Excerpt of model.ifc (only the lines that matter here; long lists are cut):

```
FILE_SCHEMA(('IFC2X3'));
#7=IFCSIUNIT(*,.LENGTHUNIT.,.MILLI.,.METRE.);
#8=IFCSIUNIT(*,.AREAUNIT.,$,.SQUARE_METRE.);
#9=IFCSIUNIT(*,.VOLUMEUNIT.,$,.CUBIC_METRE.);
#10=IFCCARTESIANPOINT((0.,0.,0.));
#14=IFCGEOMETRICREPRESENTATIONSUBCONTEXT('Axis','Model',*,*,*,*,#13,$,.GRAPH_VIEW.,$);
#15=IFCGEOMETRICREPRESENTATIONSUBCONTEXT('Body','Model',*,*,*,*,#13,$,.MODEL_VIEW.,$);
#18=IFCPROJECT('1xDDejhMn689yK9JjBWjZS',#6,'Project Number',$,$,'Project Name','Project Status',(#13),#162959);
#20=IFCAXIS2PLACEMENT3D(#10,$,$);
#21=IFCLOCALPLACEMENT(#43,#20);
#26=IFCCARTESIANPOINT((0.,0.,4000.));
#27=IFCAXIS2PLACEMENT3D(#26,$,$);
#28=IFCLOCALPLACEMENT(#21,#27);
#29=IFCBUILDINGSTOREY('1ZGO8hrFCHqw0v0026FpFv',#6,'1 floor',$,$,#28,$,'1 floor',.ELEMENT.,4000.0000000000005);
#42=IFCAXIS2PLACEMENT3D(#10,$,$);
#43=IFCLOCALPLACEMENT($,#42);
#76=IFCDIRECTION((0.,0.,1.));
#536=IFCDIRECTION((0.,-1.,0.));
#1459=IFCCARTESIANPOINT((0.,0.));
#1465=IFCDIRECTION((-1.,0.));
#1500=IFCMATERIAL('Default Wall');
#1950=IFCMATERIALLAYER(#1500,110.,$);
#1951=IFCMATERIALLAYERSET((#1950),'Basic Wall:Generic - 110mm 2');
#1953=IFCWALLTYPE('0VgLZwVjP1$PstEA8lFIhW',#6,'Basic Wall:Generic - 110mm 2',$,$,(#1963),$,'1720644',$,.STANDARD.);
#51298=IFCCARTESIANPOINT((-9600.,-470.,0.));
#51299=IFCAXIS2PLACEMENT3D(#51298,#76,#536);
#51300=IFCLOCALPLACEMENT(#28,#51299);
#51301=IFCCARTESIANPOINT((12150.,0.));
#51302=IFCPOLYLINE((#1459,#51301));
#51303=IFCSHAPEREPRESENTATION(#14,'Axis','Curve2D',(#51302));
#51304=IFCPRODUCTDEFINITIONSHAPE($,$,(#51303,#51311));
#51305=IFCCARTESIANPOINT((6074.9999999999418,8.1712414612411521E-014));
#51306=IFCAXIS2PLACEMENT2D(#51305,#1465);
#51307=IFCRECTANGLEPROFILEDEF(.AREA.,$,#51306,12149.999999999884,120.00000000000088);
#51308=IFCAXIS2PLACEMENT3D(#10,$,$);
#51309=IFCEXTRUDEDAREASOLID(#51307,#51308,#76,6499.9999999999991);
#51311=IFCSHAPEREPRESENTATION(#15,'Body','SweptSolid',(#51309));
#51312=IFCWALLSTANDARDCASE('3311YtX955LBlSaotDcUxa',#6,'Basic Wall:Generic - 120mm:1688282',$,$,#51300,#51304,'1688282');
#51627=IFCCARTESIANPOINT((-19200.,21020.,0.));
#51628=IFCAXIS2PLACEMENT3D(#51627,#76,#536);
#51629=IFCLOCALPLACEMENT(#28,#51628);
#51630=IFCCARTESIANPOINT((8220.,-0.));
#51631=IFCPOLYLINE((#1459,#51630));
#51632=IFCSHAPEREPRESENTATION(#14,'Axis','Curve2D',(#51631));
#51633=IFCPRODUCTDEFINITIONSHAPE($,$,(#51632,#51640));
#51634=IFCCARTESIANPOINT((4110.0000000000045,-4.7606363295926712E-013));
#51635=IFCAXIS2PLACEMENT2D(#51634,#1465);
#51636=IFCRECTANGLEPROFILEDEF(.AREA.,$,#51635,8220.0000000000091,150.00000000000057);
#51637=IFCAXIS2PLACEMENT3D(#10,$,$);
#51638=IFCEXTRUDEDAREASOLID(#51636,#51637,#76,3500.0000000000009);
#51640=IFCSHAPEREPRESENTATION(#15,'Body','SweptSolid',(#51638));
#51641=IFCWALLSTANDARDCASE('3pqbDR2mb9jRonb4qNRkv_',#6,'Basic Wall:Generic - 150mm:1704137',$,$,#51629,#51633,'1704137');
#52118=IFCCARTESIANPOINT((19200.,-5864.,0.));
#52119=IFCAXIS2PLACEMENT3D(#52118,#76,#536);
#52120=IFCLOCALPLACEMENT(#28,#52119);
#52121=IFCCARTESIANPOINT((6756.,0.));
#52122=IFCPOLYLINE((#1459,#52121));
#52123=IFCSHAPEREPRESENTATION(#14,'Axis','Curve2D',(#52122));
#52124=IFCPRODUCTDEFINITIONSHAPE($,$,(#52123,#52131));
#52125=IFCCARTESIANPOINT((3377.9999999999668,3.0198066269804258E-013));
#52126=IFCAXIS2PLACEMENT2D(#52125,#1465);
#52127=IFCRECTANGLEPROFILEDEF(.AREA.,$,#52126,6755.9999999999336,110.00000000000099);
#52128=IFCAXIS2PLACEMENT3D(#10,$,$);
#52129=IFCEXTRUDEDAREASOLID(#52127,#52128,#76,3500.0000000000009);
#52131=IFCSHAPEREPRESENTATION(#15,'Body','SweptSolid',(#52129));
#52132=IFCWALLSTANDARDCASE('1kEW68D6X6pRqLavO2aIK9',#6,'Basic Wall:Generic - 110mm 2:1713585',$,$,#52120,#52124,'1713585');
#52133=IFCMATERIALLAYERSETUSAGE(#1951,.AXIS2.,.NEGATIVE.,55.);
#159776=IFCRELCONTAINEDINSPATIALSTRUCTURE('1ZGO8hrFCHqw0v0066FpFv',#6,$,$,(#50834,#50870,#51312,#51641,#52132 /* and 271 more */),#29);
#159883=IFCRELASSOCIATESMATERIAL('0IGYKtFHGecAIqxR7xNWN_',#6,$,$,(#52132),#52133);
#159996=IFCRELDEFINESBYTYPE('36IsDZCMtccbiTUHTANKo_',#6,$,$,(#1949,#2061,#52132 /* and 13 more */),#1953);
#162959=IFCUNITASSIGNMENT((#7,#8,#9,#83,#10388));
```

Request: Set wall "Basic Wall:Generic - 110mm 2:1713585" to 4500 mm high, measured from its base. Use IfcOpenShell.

```python
import ifcopenshell
import ifcopenshell.geom
import ifcopenshell.util.representation
import ifcopenshell.util.shape
import ifcopenshell.util.unit

model = ifcopenshell.open("model.ifc")
unit_scale = ifcopenshell.util.unit.calculate_unit_scale(model)
settings = ifcopenshell.geom.settings()


def volume(element):
    """Net volume in cubic metres, openings subtracted."""
    shape = ifcopenshell.geom.create_shape(settings, element)
    return ifcopenshell.util.shape.get_volume(shape.geometry)


wall = model.by_guid("1kEW68D6X6pRqLavO2aIK9")
before = volume(wall)

body = ifcopenshell.util.representation.get_representation(wall, "Model", "Body")
solid = body.Items[0]
old_height = solid.Depth
solid.Depth = 4.5 / unit_scale
after = volume(wall)

print(f"height {old_height:g} -> {solid.Depth:g}, volume {before:.3f} -> {after:.3f} m3")

model.write("model_v2.ifc")
```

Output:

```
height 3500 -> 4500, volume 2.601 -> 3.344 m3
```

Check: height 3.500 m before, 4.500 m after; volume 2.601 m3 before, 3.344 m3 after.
